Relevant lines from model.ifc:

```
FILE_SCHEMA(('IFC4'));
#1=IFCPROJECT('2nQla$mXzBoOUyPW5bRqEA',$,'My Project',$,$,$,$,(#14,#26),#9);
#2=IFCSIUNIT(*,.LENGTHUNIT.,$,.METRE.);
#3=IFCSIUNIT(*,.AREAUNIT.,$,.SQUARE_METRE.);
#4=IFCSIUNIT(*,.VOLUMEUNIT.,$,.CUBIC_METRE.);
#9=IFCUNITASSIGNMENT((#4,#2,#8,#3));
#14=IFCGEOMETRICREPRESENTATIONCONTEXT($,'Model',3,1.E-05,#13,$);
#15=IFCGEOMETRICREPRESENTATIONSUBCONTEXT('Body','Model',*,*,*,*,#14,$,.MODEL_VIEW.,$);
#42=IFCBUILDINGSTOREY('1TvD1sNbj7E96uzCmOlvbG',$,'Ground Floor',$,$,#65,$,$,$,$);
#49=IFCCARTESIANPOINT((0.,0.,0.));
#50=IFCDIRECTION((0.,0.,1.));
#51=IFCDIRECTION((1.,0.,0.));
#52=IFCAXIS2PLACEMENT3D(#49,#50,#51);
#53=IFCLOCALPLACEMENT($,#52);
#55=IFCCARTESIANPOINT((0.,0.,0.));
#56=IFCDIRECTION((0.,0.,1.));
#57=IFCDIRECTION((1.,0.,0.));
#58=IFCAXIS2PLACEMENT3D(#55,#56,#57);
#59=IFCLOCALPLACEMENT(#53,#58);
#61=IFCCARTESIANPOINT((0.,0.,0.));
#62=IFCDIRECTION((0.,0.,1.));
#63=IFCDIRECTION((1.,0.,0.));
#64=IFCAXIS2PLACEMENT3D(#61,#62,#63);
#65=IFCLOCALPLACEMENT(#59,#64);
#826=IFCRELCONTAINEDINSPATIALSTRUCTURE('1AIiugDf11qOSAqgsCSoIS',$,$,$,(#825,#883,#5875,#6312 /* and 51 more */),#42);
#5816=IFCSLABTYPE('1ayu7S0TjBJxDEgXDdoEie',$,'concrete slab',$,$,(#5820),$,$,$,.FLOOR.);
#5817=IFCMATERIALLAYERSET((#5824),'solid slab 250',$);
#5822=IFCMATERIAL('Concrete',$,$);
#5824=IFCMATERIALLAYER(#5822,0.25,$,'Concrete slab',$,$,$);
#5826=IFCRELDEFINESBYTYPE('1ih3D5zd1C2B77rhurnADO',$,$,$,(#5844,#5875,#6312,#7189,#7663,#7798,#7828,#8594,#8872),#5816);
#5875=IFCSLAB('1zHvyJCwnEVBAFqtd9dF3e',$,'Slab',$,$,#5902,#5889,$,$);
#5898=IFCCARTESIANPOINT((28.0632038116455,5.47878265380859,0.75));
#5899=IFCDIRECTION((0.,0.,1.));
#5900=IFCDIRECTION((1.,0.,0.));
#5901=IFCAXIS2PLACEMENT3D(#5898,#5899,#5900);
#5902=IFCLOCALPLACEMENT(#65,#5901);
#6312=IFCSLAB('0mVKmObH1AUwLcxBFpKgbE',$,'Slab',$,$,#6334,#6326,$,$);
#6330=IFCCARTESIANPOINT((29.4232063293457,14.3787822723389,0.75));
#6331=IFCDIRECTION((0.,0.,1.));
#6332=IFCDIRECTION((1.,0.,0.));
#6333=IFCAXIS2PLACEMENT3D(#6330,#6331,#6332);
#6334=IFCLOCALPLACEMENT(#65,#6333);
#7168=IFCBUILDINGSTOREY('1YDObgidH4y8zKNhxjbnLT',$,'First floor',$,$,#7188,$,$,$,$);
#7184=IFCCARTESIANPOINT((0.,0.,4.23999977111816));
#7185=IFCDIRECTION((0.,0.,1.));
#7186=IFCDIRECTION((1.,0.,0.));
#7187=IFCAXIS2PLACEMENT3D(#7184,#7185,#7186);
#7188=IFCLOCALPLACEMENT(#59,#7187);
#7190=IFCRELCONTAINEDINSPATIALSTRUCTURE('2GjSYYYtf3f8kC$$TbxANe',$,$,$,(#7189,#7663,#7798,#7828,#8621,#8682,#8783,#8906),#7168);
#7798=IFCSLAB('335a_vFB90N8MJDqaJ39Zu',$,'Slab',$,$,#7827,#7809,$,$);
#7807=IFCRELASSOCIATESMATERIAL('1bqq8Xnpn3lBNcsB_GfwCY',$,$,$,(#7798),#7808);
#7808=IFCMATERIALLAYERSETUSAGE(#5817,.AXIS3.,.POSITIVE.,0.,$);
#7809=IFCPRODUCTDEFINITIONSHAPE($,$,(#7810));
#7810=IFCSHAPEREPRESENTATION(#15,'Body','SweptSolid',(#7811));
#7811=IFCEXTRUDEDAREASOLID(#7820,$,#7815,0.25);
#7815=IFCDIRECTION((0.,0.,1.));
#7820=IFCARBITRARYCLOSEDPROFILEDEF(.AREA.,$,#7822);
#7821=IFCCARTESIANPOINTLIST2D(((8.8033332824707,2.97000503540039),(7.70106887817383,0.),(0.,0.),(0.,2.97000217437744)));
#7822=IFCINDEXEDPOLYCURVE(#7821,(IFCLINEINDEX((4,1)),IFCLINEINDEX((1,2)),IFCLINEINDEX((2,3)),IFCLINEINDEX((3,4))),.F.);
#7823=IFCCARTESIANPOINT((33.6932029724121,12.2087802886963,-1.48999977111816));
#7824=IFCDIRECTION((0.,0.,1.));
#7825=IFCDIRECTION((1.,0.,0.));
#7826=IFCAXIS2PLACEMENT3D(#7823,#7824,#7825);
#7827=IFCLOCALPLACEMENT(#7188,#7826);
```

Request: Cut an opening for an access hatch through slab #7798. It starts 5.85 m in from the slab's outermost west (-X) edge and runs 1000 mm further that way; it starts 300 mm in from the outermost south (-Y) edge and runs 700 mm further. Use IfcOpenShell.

```python
import numpy as np
import ifcopenshell
import ifcopenshell.api.feature
import ifcopenshell.api.geometry
import ifcopenshell.api.root
import ifcopenshell.geom
import ifcopenshell.util.placement
import ifcopenshell.util.representation
import ifcopenshell.util.shape
import ifcopenshell.util.unit

model = ifcopenshell.open("model.ifc")
unit_scale = ifcopenshell.util.unit.calculate_unit_scale(model)
settings = ifcopenshell.geom.settings()


def volume(element):
    """Net volume in cubic metres, openings subtracted."""
    shape = ifcopenshell.geom.create_shape(settings, element)
    return ifcopenshell.util.shape.get_volume(shape.geometry)


slab = model.by_id(7798)
before = volume(slab)

# Extent in the slab's own axes, in metres. The edges named are its -X and -Y sides.
slab_shape = ifcopenshell.geom.create_shape(settings, slab)
vertices = ifcopenshell.util.shape.get_vertices(slab_shape.geometry)
x_min, y_min, bottom = vertices.min(axis=0)
top = vertices[:, 2].max()

opening = ifcopenshell.api.root.create_entity(model, ifc_class="IfcOpeningElement", name="Access hatch opening", predefined_type="OPENING")
context = ifcopenshell.util.representation.get_context(model, "Model", "Body", "MODEL_VIEW")
width, depth = 1, 0.7
outline = [(0.0, 0.0), (width, 0.0), (width, depth), (0.0, depth), (0.0, 0.0)]
# Overshoot both faces by 50 mm so the cut is clean.
shape = ifcopenshell.api.geometry.add_slab_representation(
    model, context=context, depth=top - bottom + 0.1, polyline=outline
)
ifcopenshell.api.geometry.assign_representation(model, product=opening, representation=shape)

matrix = ifcopenshell.util.placement.get_local_placement(slab.ObjectPlacement)
matrix[:, 3] = matrix @ np.append(np.array([x_min + 5.85, y_min + 0.3, bottom - 0.05]) / unit_scale, 1.0)
ifcopenshell.api.geometry.edit_object_placement(model, product=opening, matrix=matrix, is_si=False)
ifcopenshell.api.feature.add_feature(model, feature=opening, element=slab)

after = volume(slab)

print(f"slab volume {before:.3f} -> {after:.3f} m3")

model.write("model-out.ifc")
```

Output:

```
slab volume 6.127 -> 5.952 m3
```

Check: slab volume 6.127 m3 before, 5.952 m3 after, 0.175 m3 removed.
